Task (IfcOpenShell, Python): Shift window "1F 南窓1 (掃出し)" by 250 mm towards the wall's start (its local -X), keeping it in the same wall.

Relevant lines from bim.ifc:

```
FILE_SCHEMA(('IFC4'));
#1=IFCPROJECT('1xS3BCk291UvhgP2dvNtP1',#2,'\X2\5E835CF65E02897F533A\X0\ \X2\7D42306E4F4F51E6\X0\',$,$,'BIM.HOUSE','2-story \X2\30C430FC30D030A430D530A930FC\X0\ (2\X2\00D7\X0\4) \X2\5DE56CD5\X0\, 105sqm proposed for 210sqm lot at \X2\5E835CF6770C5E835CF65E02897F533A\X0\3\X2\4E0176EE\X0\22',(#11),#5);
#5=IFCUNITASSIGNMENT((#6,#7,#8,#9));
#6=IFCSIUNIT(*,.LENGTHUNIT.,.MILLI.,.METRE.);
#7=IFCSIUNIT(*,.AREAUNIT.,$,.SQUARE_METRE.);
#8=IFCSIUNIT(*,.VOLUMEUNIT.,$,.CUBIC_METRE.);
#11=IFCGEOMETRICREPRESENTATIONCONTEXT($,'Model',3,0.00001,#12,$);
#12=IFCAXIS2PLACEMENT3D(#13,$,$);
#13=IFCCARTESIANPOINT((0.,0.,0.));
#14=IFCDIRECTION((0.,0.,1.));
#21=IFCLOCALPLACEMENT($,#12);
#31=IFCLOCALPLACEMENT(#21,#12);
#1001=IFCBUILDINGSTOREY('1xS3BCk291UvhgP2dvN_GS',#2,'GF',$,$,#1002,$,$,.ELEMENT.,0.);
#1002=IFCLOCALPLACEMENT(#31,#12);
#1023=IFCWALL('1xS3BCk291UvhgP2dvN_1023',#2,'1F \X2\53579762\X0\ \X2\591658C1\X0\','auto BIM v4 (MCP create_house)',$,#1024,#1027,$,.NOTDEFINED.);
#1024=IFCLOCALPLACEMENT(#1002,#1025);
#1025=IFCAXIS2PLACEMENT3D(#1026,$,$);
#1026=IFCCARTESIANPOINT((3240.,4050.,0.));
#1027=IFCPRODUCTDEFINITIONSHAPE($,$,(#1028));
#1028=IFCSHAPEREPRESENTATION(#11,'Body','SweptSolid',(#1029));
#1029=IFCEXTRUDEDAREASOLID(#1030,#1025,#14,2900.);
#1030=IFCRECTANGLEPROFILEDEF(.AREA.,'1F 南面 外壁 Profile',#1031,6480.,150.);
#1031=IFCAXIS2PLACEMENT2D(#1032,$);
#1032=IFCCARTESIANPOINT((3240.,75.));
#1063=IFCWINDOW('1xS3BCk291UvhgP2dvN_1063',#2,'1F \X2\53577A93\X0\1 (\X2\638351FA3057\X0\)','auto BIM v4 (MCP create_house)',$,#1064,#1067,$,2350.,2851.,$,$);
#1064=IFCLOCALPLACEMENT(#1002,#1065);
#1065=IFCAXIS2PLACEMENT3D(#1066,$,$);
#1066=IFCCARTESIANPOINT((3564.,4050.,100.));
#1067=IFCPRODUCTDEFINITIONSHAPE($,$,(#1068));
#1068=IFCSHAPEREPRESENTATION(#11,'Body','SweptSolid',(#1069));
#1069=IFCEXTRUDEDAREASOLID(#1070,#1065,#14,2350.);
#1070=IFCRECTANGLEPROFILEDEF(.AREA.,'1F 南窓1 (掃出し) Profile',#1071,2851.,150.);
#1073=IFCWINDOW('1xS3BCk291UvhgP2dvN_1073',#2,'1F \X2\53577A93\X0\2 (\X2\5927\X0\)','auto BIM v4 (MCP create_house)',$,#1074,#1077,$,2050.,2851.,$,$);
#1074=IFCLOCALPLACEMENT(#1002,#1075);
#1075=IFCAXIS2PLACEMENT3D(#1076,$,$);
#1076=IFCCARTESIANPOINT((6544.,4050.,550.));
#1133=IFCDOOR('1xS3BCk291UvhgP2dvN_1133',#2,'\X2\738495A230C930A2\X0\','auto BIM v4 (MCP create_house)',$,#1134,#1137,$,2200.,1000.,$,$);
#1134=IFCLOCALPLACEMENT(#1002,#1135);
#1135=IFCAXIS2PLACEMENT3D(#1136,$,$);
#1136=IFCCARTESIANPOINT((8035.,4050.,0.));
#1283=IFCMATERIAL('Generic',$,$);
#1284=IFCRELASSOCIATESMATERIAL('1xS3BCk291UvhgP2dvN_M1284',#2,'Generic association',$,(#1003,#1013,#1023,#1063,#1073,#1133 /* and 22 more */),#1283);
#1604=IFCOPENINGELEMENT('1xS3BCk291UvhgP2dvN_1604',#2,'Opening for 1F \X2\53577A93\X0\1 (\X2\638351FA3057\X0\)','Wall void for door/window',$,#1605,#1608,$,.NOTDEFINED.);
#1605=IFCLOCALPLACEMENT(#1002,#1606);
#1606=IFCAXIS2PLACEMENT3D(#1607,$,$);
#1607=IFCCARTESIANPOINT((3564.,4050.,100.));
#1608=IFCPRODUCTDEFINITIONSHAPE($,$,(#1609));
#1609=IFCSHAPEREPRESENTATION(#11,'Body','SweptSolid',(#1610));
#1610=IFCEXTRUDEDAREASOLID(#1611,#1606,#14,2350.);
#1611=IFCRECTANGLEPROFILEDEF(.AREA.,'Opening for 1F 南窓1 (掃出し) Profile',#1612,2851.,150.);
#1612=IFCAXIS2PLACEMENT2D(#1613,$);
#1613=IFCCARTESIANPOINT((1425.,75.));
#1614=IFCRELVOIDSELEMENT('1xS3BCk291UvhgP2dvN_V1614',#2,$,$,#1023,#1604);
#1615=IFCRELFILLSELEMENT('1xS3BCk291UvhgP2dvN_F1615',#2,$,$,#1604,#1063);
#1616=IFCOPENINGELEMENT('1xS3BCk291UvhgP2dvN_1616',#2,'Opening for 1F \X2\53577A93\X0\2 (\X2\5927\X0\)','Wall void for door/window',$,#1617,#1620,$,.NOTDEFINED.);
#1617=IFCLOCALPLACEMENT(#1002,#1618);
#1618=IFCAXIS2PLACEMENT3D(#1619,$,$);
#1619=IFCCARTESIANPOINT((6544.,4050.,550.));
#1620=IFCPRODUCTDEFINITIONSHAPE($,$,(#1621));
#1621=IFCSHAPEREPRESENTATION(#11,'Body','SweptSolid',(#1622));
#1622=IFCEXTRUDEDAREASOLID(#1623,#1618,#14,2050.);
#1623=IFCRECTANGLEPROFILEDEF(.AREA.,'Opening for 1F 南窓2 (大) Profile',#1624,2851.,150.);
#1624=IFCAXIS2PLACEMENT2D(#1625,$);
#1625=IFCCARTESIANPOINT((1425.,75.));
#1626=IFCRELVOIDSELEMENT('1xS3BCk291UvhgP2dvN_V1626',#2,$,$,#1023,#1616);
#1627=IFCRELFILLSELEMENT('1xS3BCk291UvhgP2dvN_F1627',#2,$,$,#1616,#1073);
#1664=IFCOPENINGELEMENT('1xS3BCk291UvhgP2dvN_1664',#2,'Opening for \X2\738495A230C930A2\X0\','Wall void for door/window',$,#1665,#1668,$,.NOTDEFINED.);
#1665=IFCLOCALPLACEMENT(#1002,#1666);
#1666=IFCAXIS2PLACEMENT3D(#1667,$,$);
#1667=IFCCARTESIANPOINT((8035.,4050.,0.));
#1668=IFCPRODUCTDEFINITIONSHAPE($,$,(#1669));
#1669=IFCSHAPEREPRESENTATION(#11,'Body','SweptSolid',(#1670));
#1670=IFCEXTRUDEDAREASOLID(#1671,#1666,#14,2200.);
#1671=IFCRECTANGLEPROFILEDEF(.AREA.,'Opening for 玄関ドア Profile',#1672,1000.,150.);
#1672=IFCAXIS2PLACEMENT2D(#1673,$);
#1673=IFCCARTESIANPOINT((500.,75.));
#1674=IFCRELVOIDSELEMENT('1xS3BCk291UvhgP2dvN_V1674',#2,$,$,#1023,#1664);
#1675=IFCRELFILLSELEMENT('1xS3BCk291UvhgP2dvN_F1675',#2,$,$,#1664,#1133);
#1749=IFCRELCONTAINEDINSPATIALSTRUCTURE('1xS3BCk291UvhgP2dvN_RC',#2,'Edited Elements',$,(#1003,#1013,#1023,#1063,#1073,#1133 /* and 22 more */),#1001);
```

```python
import ifcopenshell
import ifcopenshell.api.geometry
import ifcopenshell.util.placement
import ifcopenshell.util.unit

model = ifcopenshell.open("bim.ifc")
unit_scale = ifcopenshell.util.unit.calculate_unit_scale(model)

window = model.by_id(1063)
opening = window.FillsVoids[0].RelatingOpeningElement
wall = opening.VoidsElements[0].RelatingBuildingElement

wall_matrix = ifcopenshell.util.placement.get_local_placement(wall.ObjectPlacement)
shift = wall_matrix[:3, 0] * -0.25 / unit_scale
before = ifcopenshell.util.placement.get_local_placement(window.ObjectPlacement)[:3, 3].copy()

# The window is not placed relative to its opening, so move both.
for product in (opening, window):
    matrix = ifcopenshell.util.placement.get_local_placement(product.ObjectPlacement)
    matrix[:3, 3] += shift
    ifcopenshell.api.geometry.edit_object_placement(model, product=product, matrix=matrix, is_si=False)

after = ifcopenshell.util.placement.get_local_placement(window.ObjectPlacement)[:3, 3]
print("window moved by", (after - before).round(3) + 0.0)

model.write("bim_edited.ifc")
```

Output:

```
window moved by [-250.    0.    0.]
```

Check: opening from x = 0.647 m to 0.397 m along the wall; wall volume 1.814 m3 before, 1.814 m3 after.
